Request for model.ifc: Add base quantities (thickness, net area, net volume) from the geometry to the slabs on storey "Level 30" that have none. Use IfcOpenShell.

First a look at what the model holds.

```python
import ifcopenshell
import ifcopenshell.util.element
import ifcopenshell.util.unit

model = ifcopenshell.open("model.ifc")
print(model.schema)
for unit_type in ("LENGTHUNIT", "AREAUNIT", "VOLUMEUNIT"):
    print(unit_type, ifcopenshell.util.unit.calculate_unit_scale(model, unit_type))
storey = next(s for s in model.by_type("IfcBuildingStorey") if s.Name == "Level 30")
slabs = [e for e in ifcopenshell.util.element.get_decomposition(storey) if e.is_a("IfcSlab")]
for e in sorted(slabs, key=lambda e: e.id()):
    print(e.id(), e.is_a(), e.Name, list(ifcopenshell.util.element.get_psets(e, qtos_only=True)), sep=" | ")
```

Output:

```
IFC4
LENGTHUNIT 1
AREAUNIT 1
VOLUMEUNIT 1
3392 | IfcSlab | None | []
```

```python
import ifcopenshell
import ifcopenshell.api.pset
import ifcopenshell.geom
import ifcopenshell.util.element
import ifcopenshell.util.shape
import ifcopenshell.util.unit

model = ifcopenshell.open("model.ifc")
unit_scale = ifcopenshell.util.unit.calculate_unit_scale(model)
area_scale = ifcopenshell.util.unit.calculate_unit_scale(model, "AREAUNIT")
volume_scale = ifcopenshell.util.unit.calculate_unit_scale(model, "VOLUMEUNIT")
settings = ifcopenshell.geom.settings()

storey = next(s for s in model.by_type("IfcBuildingStorey") if s.Name == "Level 30")
slabs = [e for e in ifcopenshell.util.element.get_decomposition(storey) if e.is_a("IfcSlab")]

for e in sorted(slabs, key=lambda e: e.id()):
    if ifcopenshell.util.element.get_psets(e, qtos_only=True, should_inherit=False):
        continue
    # Geometry comes back in metres, in the element's own axes.
    shape = ifcopenshell.geom.create_shape(settings, e)
    values = {
        "Width": ifcopenshell.util.shape.get_z(shape.geometry) / unit_scale,
        "NetArea": ifcopenshell.util.shape.get_footprint_area(shape.geometry) / area_scale,
        "NetVolume": ifcopenshell.util.shape.get_volume(shape.geometry) / volume_scale,
    }
    qto = ifcopenshell.api.pset.add_qto(model, product=e, name="Qto_SlabBaseQuantities")
    ifcopenshell.api.pset.edit_qto(model, qto=qto, properties=values)
    print(e.id(), {k: round(v, 3) for k, v in values.items()})

model.write("model_updated.ifc")
```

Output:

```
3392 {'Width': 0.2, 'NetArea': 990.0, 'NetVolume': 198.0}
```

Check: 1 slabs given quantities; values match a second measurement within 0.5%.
